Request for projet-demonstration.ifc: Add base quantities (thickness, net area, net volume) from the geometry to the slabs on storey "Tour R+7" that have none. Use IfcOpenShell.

First a look at what the model holds.

```python
import ifcopenshell
import ifcopenshell.util.element
import ifcopenshell.util.unit

model = ifcopenshell.open("projet-demonstration.ifc")
print(model.schema)
for unit_type in ("LENGTHUNIT", "AREAUNIT", "VOLUMEUNIT"):
    print(unit_type, ifcopenshell.util.unit.calculate_unit_scale(model, unit_type))
storey = next(s for s in model.by_type("IfcBuildingStorey") if s.Name == "Tour R+7")
slabs = [e for e in ifcopenshell.util.element.get_decomposition(storey) if e.is_a("IfcSlab")]
for e in sorted(slabs, key=lambda e: e.id()):
    print(e.id(), e.is_a(), e.Name, list(ifcopenshell.util.element.get_psets(e, qtos_only=True)), sep=" | ")
```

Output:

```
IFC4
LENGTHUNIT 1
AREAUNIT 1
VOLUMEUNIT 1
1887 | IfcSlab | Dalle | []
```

```python
import ifcopenshell
import ifcopenshell.api.pset
import ifcopenshell.geom
import ifcopenshell.util.element
import ifcopenshell.util.shape
import ifcopenshell.util.unit

model = ifcopenshell.open("projet-demonstration.ifc")
unit_scale = ifcopenshell.util.unit.calculate_unit_scale(model)
area_scale = ifcopenshell.util.unit.calculate_unit_scale(model, "AREAUNIT")
volume_scale = ifcopenshell.util.unit.calculate_unit_scale(model, "VOLUMEUNIT")
settings = ifcopenshell.geom.settings()

storey = next(s for s in model.by_type("IfcBuildingStorey") if s.Name == "Tour R+7")
slabs = [e for e in ifcopenshell.util.element.get_decomposition(storey) if e.is_a("IfcSlab")]

for e in sorted(slabs, key=lambda e: e.id()):
    if ifcopenshell.util.element.get_psets(e, qtos_only=True, should_inherit=False):
        continue
    # Geometry comes back in metres, in the element's own axes.
    shape = ifcopenshell.geom.create_shape(settings, e)
    values = {
        "Width": ifcopenshell.util.shape.get_z(shape.geometry) / unit_scale,
        "NetArea": ifcopenshell.util.shape.get_footprint_area(shape.geometry) / area_scale,
        "NetVolume": ifcopenshell.util.shape.get_volume(shape.geometry) / volume_scale,
    }
    qto = ifcopenshell.api.pset.add_qto(model, product=e, name="Qto_SlabBaseQuantities")
    ifcopenshell.api.pset.edit_qto(model, qto=qto, properties=values)
    print(e.id(), {k: round(v, 3) for k, v in values.items()})

model.write("projet-demonstration_updated.ifc")
```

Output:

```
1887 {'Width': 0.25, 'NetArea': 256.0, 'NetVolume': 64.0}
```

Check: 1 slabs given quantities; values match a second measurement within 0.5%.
